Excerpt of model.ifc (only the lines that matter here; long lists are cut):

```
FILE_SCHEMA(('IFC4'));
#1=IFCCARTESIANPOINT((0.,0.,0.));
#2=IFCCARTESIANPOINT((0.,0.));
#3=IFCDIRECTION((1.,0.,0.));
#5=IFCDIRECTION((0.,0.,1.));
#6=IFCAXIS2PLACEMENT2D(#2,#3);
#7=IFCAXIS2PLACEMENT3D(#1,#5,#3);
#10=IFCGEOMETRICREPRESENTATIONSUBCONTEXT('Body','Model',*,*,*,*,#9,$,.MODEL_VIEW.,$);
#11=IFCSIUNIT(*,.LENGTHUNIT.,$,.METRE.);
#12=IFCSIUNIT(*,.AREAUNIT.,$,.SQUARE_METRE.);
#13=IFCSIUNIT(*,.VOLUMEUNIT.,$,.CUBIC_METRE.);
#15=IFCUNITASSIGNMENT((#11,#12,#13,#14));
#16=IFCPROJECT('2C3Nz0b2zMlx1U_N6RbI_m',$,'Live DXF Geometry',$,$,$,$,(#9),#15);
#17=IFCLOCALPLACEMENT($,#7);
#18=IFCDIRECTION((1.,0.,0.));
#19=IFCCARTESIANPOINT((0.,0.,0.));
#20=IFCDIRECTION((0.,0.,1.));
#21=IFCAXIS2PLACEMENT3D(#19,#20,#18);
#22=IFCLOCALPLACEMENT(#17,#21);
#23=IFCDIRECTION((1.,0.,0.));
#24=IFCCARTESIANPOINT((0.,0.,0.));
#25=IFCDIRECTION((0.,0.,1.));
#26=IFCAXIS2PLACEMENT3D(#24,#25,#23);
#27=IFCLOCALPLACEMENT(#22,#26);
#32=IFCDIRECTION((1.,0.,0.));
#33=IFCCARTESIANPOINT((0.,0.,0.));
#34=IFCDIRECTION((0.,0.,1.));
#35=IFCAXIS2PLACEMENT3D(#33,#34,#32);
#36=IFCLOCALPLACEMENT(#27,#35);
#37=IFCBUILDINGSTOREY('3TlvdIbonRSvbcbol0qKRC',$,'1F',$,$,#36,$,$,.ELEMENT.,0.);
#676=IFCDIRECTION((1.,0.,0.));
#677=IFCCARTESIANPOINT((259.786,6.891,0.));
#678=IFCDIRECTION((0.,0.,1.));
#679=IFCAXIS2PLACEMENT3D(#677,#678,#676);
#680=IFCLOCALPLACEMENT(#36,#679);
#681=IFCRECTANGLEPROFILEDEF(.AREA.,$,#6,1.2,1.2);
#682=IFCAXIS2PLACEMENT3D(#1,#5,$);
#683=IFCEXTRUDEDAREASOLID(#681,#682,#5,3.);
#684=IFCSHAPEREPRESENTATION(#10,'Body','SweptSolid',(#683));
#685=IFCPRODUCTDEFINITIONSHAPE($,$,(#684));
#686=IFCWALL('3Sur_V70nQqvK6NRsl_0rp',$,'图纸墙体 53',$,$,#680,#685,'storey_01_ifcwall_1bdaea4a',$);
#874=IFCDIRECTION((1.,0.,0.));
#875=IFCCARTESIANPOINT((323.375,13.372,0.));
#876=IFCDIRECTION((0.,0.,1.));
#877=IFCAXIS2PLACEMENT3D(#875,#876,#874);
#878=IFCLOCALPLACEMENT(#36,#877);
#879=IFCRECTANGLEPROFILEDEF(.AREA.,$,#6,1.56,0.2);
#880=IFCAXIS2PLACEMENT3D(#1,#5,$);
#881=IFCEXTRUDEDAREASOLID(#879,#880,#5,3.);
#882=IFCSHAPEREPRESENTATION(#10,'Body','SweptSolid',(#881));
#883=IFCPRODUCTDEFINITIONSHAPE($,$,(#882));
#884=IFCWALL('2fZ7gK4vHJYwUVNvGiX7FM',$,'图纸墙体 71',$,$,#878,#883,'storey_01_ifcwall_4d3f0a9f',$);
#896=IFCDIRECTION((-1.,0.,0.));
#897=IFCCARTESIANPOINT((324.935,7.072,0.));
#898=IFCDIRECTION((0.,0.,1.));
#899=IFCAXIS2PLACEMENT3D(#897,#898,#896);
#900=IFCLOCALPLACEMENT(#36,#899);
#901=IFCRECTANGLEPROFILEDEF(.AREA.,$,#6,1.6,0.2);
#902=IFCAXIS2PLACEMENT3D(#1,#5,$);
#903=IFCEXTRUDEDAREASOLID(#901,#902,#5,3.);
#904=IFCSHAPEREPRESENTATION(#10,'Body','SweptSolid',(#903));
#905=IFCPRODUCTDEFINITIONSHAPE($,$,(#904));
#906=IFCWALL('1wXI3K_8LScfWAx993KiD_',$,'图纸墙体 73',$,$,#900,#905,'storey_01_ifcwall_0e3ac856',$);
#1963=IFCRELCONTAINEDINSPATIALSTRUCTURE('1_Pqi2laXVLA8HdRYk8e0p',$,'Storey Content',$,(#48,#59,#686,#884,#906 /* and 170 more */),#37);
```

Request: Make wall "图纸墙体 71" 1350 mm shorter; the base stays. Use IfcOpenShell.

```python
import ifcopenshell
import ifcopenshell.geom
import ifcopenshell.util.representation
import ifcopenshell.util.shape

model = ifcopenshell.open("model.ifc")
settings = ifcopenshell.geom.settings()


def volume(element):
    """Net volume in cubic metres, openings subtracted."""
    shape = ifcopenshell.geom.create_shape(settings, element)
    return ifcopenshell.util.shape.get_volume(shape.geometry)


wall = model.by_guid("2fZ7gK4vHJYwUVNvGiX7FM")
before = volume(wall)

body = ifcopenshell.util.representation.get_representation(wall, "Model", "Body")
solid = body.Items[0]
old_height = solid.Depth
solid.Depth -= 1.35
after = volume(wall)

print(f"height {old_height:g} -> {solid.Depth:g}, volume {before:.3f} -> {after:.3f} m3")

model.write("model_updated.ifc")
```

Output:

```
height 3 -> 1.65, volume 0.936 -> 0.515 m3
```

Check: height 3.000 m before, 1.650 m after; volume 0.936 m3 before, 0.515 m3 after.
